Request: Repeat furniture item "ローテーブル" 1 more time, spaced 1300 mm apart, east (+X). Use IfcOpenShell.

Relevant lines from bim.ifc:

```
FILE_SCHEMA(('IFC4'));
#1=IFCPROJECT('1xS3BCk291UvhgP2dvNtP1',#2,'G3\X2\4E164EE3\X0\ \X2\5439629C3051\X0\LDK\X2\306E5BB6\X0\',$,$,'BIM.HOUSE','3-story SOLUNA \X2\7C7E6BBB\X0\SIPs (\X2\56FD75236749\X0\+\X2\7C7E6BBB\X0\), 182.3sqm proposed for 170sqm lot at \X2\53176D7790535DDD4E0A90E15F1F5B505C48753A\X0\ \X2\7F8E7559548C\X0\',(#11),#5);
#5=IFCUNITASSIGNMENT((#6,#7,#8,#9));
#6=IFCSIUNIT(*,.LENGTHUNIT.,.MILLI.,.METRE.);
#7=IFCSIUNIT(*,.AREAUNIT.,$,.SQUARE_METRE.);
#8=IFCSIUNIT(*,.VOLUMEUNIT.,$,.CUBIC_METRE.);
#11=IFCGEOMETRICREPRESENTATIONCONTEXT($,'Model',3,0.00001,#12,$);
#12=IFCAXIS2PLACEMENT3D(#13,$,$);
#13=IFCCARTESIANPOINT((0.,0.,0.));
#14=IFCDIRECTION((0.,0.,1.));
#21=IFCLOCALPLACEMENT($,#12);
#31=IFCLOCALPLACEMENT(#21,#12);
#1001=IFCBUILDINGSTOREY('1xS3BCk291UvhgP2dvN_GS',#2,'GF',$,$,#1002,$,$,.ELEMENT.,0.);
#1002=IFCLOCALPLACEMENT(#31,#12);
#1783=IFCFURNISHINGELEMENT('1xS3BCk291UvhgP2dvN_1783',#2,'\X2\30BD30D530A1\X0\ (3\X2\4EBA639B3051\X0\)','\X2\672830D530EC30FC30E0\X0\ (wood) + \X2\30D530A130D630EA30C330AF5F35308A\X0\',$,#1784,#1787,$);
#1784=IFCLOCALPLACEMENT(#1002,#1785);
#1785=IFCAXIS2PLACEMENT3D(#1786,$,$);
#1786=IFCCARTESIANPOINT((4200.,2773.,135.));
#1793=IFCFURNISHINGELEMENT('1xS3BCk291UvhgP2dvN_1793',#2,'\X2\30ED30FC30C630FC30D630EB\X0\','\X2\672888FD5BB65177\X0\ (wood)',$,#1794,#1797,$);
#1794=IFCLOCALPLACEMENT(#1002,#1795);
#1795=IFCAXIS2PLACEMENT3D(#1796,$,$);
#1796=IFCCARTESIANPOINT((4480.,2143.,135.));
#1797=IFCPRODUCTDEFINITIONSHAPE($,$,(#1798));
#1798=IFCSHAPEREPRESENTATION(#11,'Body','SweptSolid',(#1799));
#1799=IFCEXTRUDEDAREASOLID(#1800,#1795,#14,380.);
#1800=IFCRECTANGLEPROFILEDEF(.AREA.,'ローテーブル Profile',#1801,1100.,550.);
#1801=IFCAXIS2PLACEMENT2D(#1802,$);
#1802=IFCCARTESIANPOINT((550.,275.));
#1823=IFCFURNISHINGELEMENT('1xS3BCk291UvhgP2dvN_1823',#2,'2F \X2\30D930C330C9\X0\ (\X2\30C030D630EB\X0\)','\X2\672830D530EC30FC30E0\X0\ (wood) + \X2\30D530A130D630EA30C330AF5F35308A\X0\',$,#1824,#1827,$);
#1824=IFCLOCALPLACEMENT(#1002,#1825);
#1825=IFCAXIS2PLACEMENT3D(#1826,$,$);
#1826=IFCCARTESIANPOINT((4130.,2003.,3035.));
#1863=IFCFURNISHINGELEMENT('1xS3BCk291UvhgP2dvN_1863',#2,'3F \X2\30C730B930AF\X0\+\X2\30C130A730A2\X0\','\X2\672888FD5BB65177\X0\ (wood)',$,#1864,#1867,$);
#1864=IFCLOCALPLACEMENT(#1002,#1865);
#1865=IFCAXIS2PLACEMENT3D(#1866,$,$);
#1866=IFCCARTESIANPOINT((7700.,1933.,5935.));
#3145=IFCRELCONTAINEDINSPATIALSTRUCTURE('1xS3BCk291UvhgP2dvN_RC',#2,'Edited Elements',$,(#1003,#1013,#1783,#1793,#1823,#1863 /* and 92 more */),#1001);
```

```python
import numpy as np
import ifcopenshell
import ifcopenshell.api.geometry
import ifcopenshell.api.root
import ifcopenshell.util.element
import ifcopenshell.util.placement

model = ifcopenshell.open("bim.ifc")


def reuse_history(source, copy):
    """copy_class also copies each property set's owner history, people and application; keep the originals."""
    for rel in copy.IsDefinedBy:
        if rel.is_a("IfcRelDefinesByProperties") and (history := rel.RelatingPropertyDefinition.OwnerHistory):
            rel.RelatingPropertyDefinition.OwnerHistory = source.OwnerHistory
            ifcopenshell.util.element.remove_deep2(model, history)


source = model.by_id(1793)
base = ifcopenshell.util.placement.get_local_placement(source.ObjectPlacement)
step = np.array([1.0, 0.0, 0.0]) * 1300.0

for i in range(1, 2):
    copy = ifcopenshell.api.root.copy_class(model, product=source)
    copy.Representation = ifcopenshell.util.element.copy_deep(
        model, source.Representation, exclude=["IfcGeometricRepresentationContext", "IfcRepresentationMap"]
    )
    reuse_history(source, copy)
    matrix = base.copy()
    matrix[:3, 3] += i * step
    print("added at", matrix[:3, 3].round(3) + 0.0)
    ifcopenshell.api.geometry.edit_object_placement(model, product=copy, matrix=matrix, is_si=False)

model.write("bim_edited.ifc")
```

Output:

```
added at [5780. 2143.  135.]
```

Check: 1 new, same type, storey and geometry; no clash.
